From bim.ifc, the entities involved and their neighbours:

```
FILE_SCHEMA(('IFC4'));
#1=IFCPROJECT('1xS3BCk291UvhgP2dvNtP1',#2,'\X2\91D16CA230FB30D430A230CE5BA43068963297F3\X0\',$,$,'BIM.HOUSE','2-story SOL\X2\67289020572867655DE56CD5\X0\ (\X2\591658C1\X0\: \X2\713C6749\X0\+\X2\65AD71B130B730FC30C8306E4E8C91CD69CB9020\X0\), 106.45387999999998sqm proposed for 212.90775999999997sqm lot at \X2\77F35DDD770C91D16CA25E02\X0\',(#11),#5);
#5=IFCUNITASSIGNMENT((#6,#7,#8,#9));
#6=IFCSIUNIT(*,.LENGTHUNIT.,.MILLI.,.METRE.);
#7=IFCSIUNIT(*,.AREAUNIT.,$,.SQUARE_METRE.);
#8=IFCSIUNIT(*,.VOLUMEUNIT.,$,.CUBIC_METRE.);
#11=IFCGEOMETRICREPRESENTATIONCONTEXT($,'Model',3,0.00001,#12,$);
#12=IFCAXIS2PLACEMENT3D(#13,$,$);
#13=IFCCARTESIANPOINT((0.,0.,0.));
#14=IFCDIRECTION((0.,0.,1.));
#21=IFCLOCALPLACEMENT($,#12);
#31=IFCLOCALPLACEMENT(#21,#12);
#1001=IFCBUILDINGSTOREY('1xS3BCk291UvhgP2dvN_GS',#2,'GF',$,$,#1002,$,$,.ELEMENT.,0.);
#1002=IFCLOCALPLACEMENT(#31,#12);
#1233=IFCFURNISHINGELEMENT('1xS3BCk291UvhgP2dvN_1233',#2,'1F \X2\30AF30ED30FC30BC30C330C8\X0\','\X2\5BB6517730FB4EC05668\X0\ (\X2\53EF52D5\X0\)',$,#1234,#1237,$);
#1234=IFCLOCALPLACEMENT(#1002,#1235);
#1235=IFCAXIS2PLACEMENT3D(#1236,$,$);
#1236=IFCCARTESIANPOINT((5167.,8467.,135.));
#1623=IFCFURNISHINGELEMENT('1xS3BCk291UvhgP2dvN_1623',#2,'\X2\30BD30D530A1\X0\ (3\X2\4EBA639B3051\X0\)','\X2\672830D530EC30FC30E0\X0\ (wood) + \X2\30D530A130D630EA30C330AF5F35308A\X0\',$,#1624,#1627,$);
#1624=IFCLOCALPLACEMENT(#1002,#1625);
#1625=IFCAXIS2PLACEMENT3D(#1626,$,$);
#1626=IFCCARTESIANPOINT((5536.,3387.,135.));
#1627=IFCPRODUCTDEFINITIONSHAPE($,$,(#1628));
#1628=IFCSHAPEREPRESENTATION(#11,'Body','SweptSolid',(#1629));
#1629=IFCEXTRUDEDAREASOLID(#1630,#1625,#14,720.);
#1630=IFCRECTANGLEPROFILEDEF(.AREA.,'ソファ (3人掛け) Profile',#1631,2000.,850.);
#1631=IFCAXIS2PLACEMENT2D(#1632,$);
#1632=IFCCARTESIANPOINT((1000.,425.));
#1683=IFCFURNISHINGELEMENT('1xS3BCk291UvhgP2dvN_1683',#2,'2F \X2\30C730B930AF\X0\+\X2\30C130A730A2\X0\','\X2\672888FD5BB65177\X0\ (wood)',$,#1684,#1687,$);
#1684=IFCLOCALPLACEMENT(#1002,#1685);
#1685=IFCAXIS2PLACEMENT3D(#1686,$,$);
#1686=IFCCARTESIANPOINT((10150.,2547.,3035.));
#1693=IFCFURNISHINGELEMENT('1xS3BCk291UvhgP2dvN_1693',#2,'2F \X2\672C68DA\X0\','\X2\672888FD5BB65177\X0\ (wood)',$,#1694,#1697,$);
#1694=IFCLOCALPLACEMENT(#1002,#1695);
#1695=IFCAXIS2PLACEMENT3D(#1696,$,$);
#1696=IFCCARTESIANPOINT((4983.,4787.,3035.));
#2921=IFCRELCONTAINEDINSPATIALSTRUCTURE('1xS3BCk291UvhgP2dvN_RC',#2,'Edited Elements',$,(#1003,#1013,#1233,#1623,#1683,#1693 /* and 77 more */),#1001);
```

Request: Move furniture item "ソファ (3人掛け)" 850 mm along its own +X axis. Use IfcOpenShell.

```python
import ifcopenshell
import ifcopenshell.api.geometry
import ifcopenshell.util.placement
import ifcopenshell.util.unit

model = ifcopenshell.open("bim.ifc")
unit_scale = ifcopenshell.util.unit.calculate_unit_scale(model)

item = model.by_guid("1xS3BCk291UvhgP2dvN_1623")
matrix = ifcopenshell.util.placement.get_local_placement(item.ObjectPlacement)
matrix[:3, 3] += matrix[:3, 0] * 0.85 / unit_scale
ifcopenshell.api.geometry.edit_object_placement(model, product=item, matrix=matrix, is_si=False)

print(ifcopenshell.util.placement.get_local_placement(item.ObjectPlacement).round(3) + 0.0)

model.write("bim_rev.ifc")
```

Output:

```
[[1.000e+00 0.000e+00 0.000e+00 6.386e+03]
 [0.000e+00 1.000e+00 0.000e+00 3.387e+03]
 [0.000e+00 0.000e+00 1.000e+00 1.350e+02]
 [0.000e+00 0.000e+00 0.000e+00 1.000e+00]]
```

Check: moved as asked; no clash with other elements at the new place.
